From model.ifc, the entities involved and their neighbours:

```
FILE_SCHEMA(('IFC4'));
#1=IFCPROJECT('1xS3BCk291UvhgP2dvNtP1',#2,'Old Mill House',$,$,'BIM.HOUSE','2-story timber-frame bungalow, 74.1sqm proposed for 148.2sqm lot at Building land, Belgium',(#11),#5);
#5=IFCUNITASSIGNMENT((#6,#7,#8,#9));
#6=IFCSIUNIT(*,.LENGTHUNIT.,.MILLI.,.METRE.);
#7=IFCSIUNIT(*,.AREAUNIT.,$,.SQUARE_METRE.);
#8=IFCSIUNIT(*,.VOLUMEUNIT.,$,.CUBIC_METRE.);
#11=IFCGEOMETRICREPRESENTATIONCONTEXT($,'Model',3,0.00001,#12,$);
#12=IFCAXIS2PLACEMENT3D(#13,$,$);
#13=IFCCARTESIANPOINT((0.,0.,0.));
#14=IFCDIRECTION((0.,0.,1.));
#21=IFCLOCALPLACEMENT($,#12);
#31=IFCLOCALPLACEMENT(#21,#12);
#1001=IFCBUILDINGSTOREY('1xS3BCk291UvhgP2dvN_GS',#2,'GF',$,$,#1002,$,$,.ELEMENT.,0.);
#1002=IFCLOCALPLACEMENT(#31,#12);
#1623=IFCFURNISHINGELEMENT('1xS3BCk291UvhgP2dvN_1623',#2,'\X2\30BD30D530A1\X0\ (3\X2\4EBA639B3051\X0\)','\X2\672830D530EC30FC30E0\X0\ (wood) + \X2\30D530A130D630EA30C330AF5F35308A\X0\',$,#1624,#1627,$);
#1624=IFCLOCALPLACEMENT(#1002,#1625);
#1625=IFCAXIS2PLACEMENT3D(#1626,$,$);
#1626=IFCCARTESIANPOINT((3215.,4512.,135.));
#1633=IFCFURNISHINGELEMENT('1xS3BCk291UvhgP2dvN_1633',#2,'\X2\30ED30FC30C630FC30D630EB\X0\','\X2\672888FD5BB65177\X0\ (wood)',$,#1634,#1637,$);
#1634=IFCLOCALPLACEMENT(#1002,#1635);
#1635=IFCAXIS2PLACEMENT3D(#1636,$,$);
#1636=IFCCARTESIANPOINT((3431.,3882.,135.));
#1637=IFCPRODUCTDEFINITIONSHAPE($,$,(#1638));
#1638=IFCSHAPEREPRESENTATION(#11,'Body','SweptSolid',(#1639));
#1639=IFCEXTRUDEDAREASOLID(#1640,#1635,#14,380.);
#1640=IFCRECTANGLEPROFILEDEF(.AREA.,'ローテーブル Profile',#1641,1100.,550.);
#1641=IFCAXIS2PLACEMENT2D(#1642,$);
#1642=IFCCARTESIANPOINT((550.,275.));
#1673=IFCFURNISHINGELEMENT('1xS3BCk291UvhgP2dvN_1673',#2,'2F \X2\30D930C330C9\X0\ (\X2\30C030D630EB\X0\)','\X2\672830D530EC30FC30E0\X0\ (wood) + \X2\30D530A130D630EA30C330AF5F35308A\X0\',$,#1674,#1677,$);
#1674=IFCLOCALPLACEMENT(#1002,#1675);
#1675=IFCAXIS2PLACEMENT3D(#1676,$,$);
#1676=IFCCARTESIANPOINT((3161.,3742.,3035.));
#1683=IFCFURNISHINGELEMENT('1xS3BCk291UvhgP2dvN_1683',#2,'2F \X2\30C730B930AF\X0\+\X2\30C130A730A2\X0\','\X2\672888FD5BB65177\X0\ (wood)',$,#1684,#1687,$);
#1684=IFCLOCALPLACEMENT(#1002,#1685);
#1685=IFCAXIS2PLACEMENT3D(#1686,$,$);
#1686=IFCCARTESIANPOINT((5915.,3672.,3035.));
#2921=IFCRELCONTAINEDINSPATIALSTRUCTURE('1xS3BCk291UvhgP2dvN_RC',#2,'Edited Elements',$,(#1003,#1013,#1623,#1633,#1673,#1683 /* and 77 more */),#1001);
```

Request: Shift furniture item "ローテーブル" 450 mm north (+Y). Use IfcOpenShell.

```python
import ifcopenshell
import ifcopenshell.api.geometry
import ifcopenshell.util.placement
import ifcopenshell.util.unit

model = ifcopenshell.open("model.ifc")
unit_scale = ifcopenshell.util.unit.calculate_unit_scale(model)

item = model.by_guid("1xS3BCk291UvhgP2dvN_1633")
matrix = ifcopenshell.util.placement.get_local_placement(item.ObjectPlacement)
matrix[1, 3] += 0.45 / unit_scale
ifcopenshell.api.geometry.edit_object_placement(model, product=item, matrix=matrix, is_si=False)

print(ifcopenshell.util.placement.get_local_placement(item.ObjectPlacement).round(3) + 0.0)

model.write("model_updated.ifc")
```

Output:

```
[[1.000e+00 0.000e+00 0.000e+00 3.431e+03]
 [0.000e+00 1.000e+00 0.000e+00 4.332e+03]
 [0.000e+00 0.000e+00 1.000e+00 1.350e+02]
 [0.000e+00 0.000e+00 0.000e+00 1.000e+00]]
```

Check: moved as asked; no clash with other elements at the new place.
